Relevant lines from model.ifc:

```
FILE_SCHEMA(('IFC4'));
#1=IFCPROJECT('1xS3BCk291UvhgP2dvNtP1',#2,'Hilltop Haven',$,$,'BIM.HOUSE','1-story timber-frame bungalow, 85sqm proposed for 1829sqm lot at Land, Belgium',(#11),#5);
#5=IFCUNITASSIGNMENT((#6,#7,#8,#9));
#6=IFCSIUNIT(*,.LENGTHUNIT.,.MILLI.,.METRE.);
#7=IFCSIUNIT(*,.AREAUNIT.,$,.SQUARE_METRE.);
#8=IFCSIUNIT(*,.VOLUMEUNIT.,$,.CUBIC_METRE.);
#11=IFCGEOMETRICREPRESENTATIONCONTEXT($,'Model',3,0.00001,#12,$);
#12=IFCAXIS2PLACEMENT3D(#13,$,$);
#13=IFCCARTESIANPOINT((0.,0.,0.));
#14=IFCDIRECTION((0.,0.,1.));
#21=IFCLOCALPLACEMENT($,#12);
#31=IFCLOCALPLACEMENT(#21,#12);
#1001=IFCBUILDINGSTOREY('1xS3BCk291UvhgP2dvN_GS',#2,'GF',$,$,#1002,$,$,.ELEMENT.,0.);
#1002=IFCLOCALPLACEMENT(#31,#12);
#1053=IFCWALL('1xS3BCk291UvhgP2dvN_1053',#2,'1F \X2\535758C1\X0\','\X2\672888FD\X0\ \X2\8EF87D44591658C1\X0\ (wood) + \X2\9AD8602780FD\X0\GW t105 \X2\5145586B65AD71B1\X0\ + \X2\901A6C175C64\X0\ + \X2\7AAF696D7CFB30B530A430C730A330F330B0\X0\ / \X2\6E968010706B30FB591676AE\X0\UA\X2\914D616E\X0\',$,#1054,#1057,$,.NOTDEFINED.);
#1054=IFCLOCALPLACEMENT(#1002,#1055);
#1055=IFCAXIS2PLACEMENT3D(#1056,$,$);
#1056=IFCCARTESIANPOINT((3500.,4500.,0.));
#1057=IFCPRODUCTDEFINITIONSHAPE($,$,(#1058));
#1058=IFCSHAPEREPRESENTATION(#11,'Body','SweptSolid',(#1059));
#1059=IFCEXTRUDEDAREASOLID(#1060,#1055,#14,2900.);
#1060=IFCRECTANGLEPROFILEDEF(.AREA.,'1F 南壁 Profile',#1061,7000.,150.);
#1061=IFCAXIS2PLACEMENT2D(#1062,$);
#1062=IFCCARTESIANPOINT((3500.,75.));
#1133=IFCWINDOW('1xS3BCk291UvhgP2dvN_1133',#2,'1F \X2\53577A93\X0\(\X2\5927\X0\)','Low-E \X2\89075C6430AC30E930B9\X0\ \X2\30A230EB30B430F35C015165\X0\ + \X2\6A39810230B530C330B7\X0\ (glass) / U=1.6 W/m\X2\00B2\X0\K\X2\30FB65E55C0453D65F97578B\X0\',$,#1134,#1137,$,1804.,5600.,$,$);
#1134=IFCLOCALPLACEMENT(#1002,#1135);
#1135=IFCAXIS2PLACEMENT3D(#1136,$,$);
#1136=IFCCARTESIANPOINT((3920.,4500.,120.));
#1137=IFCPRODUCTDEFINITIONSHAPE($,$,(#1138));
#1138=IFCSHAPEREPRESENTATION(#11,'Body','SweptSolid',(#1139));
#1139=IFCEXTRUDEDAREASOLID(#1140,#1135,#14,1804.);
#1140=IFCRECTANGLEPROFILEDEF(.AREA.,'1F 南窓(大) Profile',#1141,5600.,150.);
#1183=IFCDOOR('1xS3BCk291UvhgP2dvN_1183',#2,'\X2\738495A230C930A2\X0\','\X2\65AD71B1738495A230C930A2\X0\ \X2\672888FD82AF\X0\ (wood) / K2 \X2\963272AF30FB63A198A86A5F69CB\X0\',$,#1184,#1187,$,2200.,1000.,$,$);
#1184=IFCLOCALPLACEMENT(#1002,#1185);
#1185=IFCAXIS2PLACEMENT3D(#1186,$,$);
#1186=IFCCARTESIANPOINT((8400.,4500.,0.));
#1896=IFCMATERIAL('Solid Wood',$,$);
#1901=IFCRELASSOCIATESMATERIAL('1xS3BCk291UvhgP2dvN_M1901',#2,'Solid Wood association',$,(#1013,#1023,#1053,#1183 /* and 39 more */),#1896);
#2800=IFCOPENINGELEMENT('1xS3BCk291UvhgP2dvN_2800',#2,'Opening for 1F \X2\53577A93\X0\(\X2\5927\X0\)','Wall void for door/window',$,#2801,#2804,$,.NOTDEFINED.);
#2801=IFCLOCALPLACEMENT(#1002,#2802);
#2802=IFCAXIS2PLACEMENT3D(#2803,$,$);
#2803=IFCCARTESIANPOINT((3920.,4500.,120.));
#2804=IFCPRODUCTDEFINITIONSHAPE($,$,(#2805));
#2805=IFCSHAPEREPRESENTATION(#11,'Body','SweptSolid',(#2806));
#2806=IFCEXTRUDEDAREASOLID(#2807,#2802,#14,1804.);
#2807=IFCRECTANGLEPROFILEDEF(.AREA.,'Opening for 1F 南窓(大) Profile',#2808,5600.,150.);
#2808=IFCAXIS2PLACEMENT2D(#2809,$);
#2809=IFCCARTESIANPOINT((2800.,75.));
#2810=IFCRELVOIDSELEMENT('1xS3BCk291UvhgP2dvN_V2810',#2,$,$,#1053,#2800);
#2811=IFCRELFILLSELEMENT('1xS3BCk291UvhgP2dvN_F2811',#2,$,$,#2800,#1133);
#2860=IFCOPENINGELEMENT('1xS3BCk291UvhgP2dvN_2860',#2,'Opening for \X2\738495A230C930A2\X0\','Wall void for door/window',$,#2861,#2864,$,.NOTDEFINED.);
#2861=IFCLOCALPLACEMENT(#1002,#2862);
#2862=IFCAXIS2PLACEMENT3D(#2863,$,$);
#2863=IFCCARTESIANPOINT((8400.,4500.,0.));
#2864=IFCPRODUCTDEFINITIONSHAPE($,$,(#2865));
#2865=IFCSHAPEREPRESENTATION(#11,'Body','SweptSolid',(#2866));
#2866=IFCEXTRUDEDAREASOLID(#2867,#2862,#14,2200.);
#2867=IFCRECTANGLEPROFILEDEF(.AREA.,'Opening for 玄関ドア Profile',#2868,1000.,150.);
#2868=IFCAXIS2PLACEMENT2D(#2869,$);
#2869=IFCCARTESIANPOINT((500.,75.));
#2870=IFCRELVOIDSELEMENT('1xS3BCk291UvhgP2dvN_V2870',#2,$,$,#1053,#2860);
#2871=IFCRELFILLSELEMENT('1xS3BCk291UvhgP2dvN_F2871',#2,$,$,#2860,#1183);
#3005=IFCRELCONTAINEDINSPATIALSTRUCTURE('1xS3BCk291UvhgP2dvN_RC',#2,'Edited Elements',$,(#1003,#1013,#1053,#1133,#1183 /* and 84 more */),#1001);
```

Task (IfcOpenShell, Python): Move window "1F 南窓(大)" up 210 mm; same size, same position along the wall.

```python
import numpy as np
import ifcopenshell
import ifcopenshell.api.geometry
import ifcopenshell.util.placement
import ifcopenshell.util.unit

model = ifcopenshell.open("model.ifc")
unit_scale = ifcopenshell.util.unit.calculate_unit_scale(model)

window = model.by_guid("1xS3BCk291UvhgP2dvN_1133")
opening = window.FillsVoids[0].RelatingOpeningElement
dz = 0.21 / unit_scale

shift = np.array([0.0, 0.0, dz])
# The window is not placed relative to its opening, so move both.
for product in (opening, window):
    matrix = ifcopenshell.util.placement.get_local_placement(product.ObjectPlacement)
    matrix[:3, 3] += shift
    ifcopenshell.api.geometry.edit_object_placement(model, product=product, matrix=matrix, is_si=False)

print(f"moved by {dz * unit_scale:+.3f} m")

model.write("model-out.ifc")
```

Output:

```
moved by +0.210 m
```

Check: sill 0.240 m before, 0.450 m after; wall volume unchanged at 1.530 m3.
